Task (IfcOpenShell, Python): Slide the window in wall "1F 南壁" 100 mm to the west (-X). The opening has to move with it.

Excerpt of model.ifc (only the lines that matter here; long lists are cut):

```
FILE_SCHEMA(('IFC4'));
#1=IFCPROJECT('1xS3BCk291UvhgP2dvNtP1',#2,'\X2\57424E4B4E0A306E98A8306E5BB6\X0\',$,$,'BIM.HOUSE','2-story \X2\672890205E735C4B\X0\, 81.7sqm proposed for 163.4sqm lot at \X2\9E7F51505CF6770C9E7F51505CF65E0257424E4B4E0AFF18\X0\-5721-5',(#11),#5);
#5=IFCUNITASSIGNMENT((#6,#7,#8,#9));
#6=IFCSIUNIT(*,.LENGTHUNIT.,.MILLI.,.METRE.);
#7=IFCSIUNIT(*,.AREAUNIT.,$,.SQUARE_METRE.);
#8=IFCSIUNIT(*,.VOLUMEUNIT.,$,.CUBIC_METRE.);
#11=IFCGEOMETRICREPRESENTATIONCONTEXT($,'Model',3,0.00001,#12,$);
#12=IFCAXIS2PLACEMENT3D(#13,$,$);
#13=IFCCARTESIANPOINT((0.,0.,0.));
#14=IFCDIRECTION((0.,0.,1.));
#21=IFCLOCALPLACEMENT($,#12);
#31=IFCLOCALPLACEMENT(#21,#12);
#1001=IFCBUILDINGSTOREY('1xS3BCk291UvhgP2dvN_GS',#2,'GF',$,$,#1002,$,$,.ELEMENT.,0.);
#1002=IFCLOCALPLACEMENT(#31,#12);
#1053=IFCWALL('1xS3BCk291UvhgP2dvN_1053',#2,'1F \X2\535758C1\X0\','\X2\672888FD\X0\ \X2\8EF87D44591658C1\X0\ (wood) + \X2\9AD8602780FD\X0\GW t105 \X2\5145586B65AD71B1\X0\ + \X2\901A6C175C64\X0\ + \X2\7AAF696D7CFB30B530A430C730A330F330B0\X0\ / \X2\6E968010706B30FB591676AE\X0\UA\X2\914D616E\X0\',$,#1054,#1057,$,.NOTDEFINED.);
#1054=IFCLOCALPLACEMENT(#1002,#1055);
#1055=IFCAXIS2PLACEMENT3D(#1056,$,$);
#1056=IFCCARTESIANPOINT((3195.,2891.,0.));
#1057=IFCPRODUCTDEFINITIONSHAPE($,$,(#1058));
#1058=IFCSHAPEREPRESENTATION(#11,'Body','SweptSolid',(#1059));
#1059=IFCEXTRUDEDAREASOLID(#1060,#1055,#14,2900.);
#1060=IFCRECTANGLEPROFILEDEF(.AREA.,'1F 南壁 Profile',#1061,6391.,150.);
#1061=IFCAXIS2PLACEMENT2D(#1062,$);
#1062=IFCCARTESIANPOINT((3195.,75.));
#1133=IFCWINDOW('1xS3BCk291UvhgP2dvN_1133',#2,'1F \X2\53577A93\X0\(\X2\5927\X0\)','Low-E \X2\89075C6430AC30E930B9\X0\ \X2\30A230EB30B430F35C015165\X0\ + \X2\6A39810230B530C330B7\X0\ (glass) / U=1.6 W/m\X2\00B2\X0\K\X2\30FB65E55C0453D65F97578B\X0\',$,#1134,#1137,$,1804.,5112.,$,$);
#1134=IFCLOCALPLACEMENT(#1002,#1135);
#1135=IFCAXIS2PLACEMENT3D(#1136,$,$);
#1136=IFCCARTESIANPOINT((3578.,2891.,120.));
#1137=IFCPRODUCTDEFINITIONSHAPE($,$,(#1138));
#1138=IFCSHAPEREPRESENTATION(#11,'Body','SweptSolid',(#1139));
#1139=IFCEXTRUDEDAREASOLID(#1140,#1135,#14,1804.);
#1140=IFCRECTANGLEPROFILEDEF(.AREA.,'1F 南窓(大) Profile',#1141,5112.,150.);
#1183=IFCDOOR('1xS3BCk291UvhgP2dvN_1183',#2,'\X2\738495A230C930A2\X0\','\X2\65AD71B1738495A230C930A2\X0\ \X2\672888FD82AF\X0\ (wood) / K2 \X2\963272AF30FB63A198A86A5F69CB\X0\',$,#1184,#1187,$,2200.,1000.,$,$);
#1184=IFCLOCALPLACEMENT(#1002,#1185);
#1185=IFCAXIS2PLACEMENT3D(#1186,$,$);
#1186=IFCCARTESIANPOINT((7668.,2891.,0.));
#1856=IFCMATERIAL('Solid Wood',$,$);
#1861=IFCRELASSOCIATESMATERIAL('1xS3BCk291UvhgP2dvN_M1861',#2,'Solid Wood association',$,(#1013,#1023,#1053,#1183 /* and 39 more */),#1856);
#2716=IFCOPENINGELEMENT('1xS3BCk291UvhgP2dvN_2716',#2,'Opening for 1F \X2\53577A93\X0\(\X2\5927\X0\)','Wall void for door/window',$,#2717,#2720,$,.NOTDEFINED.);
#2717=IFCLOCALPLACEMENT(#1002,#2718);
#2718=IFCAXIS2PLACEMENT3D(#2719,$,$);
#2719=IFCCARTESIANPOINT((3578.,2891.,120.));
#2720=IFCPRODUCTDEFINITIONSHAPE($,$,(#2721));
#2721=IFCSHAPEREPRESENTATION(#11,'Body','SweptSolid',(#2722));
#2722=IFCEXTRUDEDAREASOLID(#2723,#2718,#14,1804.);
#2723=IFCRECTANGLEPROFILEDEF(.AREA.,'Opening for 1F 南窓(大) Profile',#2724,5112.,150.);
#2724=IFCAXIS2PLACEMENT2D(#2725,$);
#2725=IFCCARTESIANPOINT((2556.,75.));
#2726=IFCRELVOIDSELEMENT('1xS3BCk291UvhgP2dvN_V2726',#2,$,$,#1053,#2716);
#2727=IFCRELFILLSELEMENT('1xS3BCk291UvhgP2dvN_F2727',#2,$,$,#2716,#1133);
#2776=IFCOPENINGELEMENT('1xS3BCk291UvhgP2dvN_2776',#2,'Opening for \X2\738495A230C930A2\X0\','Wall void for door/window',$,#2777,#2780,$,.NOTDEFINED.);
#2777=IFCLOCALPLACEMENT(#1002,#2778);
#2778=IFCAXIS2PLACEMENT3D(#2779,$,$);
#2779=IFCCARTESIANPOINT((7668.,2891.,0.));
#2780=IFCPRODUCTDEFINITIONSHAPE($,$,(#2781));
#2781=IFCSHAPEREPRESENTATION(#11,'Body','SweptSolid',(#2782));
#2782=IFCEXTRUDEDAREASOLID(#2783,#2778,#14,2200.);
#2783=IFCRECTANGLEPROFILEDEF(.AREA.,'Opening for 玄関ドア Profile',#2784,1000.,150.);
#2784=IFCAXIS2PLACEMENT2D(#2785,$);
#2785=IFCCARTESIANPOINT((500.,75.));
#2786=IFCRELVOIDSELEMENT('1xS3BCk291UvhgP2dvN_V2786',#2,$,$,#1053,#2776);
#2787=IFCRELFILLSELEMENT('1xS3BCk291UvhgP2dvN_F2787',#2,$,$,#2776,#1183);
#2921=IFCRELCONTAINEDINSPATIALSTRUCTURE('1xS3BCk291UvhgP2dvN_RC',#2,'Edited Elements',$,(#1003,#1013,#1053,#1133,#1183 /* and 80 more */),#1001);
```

```python
import ifcopenshell
import ifcopenshell.api.geometry
import ifcopenshell.util.placement
import ifcopenshell.util.unit

model = ifcopenshell.open("model.ifc")
unit_scale = ifcopenshell.util.unit.calculate_unit_scale(model)

window = model.by_guid("1xS3BCk291UvhgP2dvN_1133")
opening = window.FillsVoids[0].RelatingOpeningElement
wall = opening.VoidsElements[0].RelatingBuildingElement

wall_matrix = ifcopenshell.util.placement.get_local_placement(wall.ObjectPlacement)
shift = wall_matrix[:3, 0] * -0.1 / unit_scale
before = ifcopenshell.util.placement.get_local_placement(window.ObjectPlacement)[:3, 3].copy()

# The window is not placed relative to its opening, so move both.
for product in (opening, window):
    matrix = ifcopenshell.util.placement.get_local_placement(product.ObjectPlacement)
    matrix[:3, 3] += shift
    ifcopenshell.api.geometry.edit_object_placement(model, product=product, matrix=matrix, is_si=False)

after = ifcopenshell.util.placement.get_local_placement(window.ObjectPlacement)[:3, 3]
print("window moved by", (after - before).round(3) + 0.0)

model.write("model_edited.ifc")
```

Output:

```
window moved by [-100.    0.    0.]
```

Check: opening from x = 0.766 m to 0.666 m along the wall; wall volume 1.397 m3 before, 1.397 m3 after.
